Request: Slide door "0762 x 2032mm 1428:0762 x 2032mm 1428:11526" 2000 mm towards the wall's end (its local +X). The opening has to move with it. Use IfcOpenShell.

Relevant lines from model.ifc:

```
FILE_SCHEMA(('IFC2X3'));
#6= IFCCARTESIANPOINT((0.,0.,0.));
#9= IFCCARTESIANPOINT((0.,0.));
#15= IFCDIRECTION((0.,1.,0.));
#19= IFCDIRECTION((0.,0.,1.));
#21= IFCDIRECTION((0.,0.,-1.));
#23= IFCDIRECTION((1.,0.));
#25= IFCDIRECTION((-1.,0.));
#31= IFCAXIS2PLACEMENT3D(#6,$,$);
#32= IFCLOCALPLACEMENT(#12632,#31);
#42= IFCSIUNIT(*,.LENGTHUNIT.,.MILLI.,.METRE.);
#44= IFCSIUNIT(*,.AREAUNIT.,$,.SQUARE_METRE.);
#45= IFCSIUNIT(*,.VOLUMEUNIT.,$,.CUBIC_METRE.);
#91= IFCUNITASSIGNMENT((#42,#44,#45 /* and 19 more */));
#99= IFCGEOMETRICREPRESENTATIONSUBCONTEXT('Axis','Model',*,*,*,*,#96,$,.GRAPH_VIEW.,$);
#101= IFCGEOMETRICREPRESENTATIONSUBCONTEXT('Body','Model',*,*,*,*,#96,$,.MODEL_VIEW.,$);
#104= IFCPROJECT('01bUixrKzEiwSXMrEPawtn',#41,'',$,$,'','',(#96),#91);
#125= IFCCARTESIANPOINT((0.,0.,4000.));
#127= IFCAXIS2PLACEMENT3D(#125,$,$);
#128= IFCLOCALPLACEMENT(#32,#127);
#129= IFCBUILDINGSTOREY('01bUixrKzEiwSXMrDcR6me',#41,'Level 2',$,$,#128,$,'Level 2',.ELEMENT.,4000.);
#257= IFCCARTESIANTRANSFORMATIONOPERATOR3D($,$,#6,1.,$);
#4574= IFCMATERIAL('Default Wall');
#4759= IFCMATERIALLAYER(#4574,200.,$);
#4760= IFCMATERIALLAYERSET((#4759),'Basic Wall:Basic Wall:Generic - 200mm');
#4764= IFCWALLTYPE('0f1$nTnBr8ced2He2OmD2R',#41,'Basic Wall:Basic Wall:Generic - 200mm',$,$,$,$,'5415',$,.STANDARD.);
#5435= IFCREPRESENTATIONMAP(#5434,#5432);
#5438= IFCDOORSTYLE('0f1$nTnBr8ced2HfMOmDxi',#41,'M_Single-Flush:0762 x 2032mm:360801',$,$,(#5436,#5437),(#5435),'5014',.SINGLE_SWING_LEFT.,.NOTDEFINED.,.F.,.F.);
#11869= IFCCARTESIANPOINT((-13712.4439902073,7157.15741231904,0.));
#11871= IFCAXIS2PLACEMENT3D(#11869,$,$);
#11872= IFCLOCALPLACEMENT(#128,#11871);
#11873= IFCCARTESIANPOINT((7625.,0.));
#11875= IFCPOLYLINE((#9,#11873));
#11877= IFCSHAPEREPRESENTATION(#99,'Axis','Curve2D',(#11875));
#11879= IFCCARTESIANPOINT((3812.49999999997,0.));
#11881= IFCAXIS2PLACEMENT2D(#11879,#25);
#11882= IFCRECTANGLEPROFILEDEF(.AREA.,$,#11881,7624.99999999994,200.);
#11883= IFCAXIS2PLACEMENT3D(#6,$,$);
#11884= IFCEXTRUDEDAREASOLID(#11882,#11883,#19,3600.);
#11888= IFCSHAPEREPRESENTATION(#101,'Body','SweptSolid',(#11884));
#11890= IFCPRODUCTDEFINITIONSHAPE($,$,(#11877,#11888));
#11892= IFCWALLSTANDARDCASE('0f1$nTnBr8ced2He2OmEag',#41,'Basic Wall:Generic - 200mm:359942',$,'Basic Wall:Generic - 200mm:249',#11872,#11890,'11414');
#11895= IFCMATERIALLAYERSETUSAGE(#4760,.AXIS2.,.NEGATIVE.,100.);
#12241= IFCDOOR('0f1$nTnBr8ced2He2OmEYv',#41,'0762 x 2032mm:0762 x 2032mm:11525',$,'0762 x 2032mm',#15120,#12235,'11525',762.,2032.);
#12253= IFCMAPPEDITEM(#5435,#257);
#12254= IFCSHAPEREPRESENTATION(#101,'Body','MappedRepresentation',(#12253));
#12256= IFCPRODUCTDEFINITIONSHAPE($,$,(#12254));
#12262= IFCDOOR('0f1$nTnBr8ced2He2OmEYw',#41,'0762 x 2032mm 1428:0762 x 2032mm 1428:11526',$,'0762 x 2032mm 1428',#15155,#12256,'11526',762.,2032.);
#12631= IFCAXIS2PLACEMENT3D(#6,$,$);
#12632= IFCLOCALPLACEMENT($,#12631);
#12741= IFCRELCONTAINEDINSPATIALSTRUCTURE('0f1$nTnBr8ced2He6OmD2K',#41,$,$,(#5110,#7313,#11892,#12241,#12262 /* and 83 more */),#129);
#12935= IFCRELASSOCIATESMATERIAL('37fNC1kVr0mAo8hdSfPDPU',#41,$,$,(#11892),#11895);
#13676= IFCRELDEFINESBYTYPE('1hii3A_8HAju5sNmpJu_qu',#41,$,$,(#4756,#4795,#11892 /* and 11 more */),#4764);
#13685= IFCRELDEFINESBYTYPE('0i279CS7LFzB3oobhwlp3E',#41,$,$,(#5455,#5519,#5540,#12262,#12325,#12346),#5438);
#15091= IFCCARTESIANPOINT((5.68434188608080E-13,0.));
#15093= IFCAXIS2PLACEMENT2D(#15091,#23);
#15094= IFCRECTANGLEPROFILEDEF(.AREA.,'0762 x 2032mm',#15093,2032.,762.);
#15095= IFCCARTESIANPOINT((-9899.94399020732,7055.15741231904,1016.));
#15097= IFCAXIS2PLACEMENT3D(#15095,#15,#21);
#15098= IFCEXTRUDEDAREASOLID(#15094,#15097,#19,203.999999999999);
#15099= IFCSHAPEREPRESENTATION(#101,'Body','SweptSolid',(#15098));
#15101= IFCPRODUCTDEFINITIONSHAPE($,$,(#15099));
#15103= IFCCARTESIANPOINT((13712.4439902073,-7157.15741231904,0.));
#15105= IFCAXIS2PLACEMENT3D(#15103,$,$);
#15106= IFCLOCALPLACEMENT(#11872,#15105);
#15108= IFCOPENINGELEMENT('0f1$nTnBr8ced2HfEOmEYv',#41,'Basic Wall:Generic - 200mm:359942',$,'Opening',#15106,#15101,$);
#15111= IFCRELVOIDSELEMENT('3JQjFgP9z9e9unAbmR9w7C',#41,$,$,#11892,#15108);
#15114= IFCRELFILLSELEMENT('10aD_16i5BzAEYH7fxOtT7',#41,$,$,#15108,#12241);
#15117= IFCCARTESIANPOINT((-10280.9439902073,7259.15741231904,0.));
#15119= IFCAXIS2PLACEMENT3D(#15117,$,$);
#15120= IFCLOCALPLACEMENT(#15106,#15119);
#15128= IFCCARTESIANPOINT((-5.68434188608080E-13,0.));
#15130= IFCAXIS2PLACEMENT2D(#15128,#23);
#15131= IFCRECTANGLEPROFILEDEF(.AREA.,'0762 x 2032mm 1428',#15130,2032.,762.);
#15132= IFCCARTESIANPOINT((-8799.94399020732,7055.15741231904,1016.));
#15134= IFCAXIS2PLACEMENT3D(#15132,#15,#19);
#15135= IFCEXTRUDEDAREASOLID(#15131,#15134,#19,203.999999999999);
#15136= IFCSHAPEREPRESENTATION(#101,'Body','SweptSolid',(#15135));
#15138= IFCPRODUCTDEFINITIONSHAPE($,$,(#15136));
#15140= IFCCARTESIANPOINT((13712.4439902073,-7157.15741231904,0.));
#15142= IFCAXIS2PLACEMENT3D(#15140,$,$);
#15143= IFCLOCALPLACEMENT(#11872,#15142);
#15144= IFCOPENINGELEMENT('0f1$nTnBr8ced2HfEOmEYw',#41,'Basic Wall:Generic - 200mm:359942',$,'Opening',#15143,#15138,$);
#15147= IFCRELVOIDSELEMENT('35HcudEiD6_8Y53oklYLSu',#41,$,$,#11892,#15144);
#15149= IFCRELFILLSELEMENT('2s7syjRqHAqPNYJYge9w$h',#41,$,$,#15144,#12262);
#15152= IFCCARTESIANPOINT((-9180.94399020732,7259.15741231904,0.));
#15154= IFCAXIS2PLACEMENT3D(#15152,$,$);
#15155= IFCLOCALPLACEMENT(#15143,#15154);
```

```python
import ifcopenshell
import ifcopenshell.api.geometry
import ifcopenshell.util.placement

model = ifcopenshell.open("model.ifc")

door = model.by_id(12262)
opening = door.FillsVoids[0].RelatingOpeningElement
wall = opening.VoidsElements[0].RelatingBuildingElement

wall_matrix = ifcopenshell.util.placement.get_local_placement(wall.ObjectPlacement)
shift = wall_matrix[:3, 0] * 2000.0
before = ifcopenshell.util.placement.get_local_placement(door.ObjectPlacement)[:3, 3].copy()

# The door is placed relative to its opening, so it follows when the opening moves.
matrix = ifcopenshell.util.placement.get_local_placement(opening.ObjectPlacement)
matrix[:3, 3] += shift
ifcopenshell.api.geometry.edit_object_placement(
    model, product=opening, matrix=matrix, is_si=False, should_transform_children=True
)

after = ifcopenshell.util.placement.get_local_placement(door.ObjectPlacement)[:3, 3]
print("door moved by", (after - before).round(3) + 0.0)

model.write("model-out.ifc")
```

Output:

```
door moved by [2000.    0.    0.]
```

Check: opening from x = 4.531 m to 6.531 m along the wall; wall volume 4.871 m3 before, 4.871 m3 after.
